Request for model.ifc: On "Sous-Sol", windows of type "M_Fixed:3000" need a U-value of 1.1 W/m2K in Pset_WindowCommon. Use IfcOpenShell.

First a look at what the model holds.

```python
import ifcopenshell
import ifcopenshell.util.element

model = ifcopenshell.open("model.ifc")
print(model.schema)
storey = next(s for s in model.by_type("IfcBuildingStorey") if s.Name == "Sous-Sol")
windows = [e for e in ifcopenshell.util.element.get_decomposition(storey) if e.is_a("IfcWindow")]
seen = {}
for e in windows:
    element_type = ifcopenshell.util.element.get_type(e)
    key = (element_type.Name if element_type != e and element_type else None, ifcopenshell.util.element.get_pset(e, "Pset_WindowCommon", "ThermalTransmittance"))
    seen[key] = seen.get(key, 0) + 1
for (name, value), count in sorted(seen.items(), key=str):
    print(count, "x", name, "|", value)
```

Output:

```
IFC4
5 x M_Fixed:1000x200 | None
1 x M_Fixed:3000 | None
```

```python
import ifcopenshell
import ifcopenshell.api.pset
import ifcopenshell.util.element

model = ifcopenshell.open("model.ifc")

storey = next(s for s in model.by_type("IfcBuildingStorey") if s.Name == "Sous-Sol")
windows = [e for e in ifcopenshell.util.element.get_decomposition(storey) if e.is_a("IfcWindow")]

count = 0
for e in windows:
    element_type = ifcopenshell.util.element.get_type(e)
    if element_type in (None, e) or element_type.Name != "M_Fixed:3000":
        continue
    # add_pset returns the element's existing set when there is one.
    pset = ifcopenshell.api.pset.add_pset(model, product=e, name="Pset_WindowCommon")
    ifcopenshell.api.pset.edit_pset(model, pset=pset, properties={"ThermalTransmittance": 1.1})
    count += 1

print(count, "windows updated")

model.write("model_rev.ifc")
```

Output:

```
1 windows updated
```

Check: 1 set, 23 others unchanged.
